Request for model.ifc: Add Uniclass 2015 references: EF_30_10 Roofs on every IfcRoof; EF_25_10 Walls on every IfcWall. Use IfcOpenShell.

First a look at what the model holds.

```python
import ifcopenshell

model = ifcopenshell.open("model.ifc")
print(model.schema)
print("classifications:", [c.Name for c in model.by_type("IfcClassification")])
for ifc_class in ("IfcDoor", "IfcRoof", "IfcStair", "IfcWall", "IfcWindow"):
    print(ifc_class, len(model.by_type(ifc_class)))
```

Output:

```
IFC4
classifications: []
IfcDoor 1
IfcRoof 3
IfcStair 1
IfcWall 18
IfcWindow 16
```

```python
import ifcopenshell
import ifcopenshell.api.classification

model = ifcopenshell.open("model.ifc")

system = ifcopenshell.api.classification.add_classification(model, classification="Uniclass 2015")

codes = {
    "IfcRoof": ("EF_30_10", "Roofs"),
    "IfcWall": ("EF_25_10", "Walls"),
}
for ifc_class, (code, name) in codes.items():
    products = model.by_type(ifc_class)
    ifcopenshell.api.classification.add_reference(
        model, products=products, classification=system, identification=code, name=name
    )
    print(code, len(products))

model.write("model_v2.ifc")
```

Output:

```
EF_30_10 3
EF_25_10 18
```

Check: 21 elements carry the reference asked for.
